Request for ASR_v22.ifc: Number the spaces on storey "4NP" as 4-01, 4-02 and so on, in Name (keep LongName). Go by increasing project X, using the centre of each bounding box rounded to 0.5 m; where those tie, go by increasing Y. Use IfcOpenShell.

First a look at what the model holds.

```python
import ifcopenshell
import ifcopenshell.util.element
import ifcopenshell.util.placement

model = ifcopenshell.open("ASR_v22.ifc")
print(model.schema)
storey = next(s for s in model.by_type("IfcBuildingStorey") if s.Name == "4NP")
spaces = [e for e in ifcopenshell.util.element.get_decomposition(storey) if e.is_a("IfcSpace")]
for e in sorted(spaces, key=lambda e: e.id()):
    origin = ifcopenshell.util.placement.get_local_placement(e.ObjectPlacement)[:3, 3]
    print(e.id(), e.Name, e.LongName, origin.round(2) + 0.0, sep=" | ")
```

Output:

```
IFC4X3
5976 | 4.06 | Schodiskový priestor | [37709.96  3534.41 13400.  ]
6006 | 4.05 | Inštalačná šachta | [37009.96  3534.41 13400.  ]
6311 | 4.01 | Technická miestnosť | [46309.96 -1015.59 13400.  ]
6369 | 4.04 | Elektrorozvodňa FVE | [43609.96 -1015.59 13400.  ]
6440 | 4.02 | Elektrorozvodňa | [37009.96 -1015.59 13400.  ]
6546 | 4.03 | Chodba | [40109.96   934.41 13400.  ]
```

```python
import ifcopenshell
import ifcopenshell.geom
import ifcopenshell.util.element
import ifcopenshell.util.shape

model = ifcopenshell.open("ASR_v22.ifc")
settings = ifcopenshell.geom.settings()
settings.set("use-world-coords", True)


def centre(element):
    shape = ifcopenshell.geom.create_shape(settings, element)
    return ifcopenshell.util.shape.get_bbox_centroid(shape.geometry)


storey = next(s for s in model.by_type("IfcBuildingStorey") if s.Name == "4NP")
spaces = [e for e in ifcopenshell.util.element.get_decomposition(storey) if e.is_a("IfcSpace")]

# Insertion points can sit at a corner or the storey origin, so sort by the geometry (in metres).
centres = {e: centre(e) for e in spaces}
spaces.sort(key=lambda e: (round(centres[e][0] / 0.5), centres[e][1]))

for i, e in enumerate(spaces, start=1):
    number = f"4-{i:02d}"
    e.Name = number
    print(e.id(), number)

model.write("ASR_v22_updated.ifc")
```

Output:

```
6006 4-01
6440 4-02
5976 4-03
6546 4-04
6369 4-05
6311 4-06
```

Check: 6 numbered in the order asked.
